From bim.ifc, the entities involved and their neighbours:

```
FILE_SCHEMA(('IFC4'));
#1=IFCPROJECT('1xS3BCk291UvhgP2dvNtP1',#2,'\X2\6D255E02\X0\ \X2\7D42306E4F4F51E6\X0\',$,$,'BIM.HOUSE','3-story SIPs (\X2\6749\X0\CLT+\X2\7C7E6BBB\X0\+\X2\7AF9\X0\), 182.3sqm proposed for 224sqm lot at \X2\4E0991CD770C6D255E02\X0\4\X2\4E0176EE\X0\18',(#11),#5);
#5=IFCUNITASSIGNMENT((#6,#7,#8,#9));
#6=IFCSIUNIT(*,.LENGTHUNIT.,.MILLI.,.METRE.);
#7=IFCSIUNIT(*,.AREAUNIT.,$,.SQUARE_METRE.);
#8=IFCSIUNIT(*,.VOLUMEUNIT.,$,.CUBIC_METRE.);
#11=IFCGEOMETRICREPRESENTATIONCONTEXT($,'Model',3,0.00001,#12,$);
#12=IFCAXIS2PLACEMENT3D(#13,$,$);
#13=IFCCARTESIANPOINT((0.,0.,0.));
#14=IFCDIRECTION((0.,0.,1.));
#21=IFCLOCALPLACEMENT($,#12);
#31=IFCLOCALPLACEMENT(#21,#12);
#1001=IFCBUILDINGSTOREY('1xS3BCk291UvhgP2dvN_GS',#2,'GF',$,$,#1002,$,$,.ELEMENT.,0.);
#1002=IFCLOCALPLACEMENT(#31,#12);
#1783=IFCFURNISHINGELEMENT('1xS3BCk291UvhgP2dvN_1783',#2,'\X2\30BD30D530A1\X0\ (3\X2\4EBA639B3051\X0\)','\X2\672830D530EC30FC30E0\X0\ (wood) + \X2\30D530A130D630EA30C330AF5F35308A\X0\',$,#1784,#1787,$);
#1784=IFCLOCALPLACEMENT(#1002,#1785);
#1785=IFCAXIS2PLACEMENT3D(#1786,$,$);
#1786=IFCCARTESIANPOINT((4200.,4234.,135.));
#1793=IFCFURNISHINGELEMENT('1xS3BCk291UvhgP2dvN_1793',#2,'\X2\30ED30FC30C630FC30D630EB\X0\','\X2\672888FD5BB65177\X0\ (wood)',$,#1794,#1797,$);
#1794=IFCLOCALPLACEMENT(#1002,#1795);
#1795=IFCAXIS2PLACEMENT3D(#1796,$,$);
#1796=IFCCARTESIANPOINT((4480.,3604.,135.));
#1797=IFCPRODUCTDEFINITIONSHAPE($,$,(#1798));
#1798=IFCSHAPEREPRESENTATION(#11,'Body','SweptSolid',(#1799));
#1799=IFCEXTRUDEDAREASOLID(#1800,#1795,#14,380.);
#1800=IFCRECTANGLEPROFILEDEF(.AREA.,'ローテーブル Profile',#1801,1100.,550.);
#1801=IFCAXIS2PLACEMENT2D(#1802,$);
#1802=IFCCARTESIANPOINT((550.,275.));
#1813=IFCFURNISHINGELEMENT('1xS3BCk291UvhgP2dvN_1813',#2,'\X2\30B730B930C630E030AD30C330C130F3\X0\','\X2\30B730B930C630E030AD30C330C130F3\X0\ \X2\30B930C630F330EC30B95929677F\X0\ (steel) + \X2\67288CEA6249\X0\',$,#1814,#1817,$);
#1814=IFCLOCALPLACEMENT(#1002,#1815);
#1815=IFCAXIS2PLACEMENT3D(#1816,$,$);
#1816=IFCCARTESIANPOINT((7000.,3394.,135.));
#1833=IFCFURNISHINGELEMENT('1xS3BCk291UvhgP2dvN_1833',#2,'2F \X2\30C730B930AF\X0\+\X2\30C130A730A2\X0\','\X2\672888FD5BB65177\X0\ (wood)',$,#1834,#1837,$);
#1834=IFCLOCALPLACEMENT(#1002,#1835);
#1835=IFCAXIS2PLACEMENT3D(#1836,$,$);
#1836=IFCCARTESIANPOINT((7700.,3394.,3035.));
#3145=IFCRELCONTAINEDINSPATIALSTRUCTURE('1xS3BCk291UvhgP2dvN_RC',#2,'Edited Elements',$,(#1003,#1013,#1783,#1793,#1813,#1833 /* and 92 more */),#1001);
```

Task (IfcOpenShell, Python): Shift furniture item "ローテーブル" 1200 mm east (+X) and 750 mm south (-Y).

```python
import ifcopenshell
import ifcopenshell.api.geometry
import ifcopenshell.util.placement
import ifcopenshell.util.unit

model = ifcopenshell.open("bim.ifc")
unit_scale = ifcopenshell.util.unit.calculate_unit_scale(model)

item = model.by_id(1793)
matrix = ifcopenshell.util.placement.get_local_placement(item.ObjectPlacement)
matrix[0, 3] += 1.2 / unit_scale
matrix[1, 3] -= 0.75 / unit_scale
ifcopenshell.api.geometry.edit_object_placement(model, product=item, matrix=matrix, is_si=False)

print(ifcopenshell.util.placement.get_local_placement(item.ObjectPlacement).round(3) + 0.0)

model.write("bim_edited.ifc")
```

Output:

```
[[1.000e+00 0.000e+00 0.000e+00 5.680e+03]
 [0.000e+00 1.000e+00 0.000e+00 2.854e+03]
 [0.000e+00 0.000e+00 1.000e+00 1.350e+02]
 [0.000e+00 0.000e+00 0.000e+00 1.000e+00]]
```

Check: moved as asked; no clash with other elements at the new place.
